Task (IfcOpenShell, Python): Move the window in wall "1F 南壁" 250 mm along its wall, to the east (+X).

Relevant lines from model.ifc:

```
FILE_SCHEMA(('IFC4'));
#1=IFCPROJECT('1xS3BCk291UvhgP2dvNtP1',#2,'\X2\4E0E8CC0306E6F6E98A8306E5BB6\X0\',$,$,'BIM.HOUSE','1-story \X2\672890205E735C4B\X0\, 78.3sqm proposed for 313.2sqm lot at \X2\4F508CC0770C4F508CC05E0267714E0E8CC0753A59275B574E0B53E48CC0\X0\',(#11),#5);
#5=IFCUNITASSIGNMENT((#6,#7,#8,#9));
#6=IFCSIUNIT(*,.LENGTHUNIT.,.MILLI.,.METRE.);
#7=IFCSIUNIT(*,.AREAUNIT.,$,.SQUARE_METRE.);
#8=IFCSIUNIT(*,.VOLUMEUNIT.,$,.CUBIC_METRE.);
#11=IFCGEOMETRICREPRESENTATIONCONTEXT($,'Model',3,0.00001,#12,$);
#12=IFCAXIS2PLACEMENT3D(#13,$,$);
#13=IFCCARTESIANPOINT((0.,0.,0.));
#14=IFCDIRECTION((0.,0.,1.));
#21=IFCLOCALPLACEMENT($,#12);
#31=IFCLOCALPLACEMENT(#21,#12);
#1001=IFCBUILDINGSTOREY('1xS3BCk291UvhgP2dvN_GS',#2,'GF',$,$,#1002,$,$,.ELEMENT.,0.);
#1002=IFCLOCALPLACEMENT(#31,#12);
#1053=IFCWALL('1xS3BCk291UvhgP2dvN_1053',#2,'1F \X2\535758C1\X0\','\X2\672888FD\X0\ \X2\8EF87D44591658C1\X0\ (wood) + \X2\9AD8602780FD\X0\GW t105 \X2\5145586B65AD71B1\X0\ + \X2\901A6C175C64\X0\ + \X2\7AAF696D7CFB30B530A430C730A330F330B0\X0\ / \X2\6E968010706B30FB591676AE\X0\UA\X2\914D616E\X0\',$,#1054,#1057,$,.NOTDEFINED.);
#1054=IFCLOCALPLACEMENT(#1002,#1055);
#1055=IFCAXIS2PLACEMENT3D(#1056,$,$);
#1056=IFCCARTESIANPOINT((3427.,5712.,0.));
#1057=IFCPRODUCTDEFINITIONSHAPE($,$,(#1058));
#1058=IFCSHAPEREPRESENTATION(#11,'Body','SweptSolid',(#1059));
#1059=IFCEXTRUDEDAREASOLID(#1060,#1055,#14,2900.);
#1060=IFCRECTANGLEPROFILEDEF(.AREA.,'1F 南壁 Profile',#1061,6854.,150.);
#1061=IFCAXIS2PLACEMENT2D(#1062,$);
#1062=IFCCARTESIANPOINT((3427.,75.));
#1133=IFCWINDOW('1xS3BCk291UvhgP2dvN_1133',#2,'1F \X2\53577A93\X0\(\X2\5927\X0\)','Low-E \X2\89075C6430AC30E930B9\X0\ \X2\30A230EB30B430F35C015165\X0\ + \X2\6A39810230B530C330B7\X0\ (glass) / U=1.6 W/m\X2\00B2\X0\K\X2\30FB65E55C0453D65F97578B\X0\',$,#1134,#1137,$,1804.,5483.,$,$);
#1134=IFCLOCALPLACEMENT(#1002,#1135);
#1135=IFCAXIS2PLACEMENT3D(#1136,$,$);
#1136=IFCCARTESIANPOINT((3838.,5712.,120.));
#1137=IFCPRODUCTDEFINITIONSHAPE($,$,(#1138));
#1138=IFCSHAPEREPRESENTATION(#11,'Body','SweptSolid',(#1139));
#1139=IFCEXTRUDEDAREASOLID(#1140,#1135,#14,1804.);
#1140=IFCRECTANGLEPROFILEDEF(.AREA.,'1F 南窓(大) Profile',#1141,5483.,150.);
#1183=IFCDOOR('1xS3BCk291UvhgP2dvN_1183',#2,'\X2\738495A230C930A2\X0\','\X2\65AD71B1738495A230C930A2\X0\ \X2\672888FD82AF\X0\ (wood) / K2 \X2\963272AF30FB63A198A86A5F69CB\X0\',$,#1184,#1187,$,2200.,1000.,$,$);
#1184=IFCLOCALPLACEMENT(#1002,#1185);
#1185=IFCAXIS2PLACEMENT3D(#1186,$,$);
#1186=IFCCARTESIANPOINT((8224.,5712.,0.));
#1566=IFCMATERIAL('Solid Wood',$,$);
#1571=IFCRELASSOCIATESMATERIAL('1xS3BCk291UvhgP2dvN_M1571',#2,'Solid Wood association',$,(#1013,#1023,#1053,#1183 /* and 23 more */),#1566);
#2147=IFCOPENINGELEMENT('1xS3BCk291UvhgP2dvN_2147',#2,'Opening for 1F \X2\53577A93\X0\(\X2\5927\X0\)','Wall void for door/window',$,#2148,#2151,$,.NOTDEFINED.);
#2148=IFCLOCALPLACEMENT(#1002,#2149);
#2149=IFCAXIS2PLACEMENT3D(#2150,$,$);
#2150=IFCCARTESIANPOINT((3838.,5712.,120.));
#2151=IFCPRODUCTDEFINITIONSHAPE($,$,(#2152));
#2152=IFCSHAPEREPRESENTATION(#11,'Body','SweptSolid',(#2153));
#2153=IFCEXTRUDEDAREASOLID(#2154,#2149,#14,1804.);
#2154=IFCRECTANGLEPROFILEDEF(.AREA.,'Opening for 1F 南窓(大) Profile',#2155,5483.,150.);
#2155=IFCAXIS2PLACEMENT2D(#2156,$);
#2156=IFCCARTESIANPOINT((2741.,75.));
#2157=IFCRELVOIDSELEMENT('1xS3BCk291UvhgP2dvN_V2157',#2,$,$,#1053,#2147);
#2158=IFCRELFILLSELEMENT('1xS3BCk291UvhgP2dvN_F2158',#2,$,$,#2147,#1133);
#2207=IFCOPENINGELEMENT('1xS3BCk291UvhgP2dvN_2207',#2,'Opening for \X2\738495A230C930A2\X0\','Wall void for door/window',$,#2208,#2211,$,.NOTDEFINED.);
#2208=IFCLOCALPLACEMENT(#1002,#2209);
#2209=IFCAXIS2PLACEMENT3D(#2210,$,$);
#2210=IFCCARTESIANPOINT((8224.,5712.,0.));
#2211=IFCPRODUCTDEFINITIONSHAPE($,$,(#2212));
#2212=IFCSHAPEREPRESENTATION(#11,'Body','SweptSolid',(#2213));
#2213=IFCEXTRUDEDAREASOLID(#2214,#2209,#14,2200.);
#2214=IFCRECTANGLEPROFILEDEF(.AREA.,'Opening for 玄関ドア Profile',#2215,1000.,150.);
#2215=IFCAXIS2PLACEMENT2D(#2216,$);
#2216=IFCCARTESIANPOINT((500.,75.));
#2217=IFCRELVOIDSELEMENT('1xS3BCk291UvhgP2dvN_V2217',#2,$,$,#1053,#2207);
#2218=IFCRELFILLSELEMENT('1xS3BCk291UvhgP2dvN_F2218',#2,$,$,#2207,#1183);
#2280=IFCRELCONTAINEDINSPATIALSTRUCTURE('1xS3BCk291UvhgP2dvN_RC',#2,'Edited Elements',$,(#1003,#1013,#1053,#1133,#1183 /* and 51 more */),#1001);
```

```python
import ifcopenshell
import ifcopenshell.api.geometry
import ifcopenshell.util.placement
import ifcopenshell.util.unit

model = ifcopenshell.open("model.ifc")
unit_scale = ifcopenshell.util.unit.calculate_unit_scale(model)

window = model.by_id(1133)
opening = window.FillsVoids[0].RelatingOpeningElement
wall = opening.VoidsElements[0].RelatingBuildingElement

wall_matrix = ifcopenshell.util.placement.get_local_placement(wall.ObjectPlacement)
shift = wall_matrix[:3, 0] * 0.25 / unit_scale
before = ifcopenshell.util.placement.get_local_placement(window.ObjectPlacement)[:3, 3].copy()

# The window is not placed relative to its opening, so move both.
for product in (opening, window):
    matrix = ifcopenshell.util.placement.get_local_placement(product.ObjectPlacement)
    matrix[:3, 3] += shift
    ifcopenshell.api.geometry.edit_object_placement(model, product=product, matrix=matrix, is_si=False)

after = ifcopenshell.util.placement.get_local_placement(window.ObjectPlacement)[:3, 3]
print("window moved by", (after - before).round(3) + 0.0)

model.write("model_edited.ifc")
```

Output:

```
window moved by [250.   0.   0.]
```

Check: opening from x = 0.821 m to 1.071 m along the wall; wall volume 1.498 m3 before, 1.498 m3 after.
